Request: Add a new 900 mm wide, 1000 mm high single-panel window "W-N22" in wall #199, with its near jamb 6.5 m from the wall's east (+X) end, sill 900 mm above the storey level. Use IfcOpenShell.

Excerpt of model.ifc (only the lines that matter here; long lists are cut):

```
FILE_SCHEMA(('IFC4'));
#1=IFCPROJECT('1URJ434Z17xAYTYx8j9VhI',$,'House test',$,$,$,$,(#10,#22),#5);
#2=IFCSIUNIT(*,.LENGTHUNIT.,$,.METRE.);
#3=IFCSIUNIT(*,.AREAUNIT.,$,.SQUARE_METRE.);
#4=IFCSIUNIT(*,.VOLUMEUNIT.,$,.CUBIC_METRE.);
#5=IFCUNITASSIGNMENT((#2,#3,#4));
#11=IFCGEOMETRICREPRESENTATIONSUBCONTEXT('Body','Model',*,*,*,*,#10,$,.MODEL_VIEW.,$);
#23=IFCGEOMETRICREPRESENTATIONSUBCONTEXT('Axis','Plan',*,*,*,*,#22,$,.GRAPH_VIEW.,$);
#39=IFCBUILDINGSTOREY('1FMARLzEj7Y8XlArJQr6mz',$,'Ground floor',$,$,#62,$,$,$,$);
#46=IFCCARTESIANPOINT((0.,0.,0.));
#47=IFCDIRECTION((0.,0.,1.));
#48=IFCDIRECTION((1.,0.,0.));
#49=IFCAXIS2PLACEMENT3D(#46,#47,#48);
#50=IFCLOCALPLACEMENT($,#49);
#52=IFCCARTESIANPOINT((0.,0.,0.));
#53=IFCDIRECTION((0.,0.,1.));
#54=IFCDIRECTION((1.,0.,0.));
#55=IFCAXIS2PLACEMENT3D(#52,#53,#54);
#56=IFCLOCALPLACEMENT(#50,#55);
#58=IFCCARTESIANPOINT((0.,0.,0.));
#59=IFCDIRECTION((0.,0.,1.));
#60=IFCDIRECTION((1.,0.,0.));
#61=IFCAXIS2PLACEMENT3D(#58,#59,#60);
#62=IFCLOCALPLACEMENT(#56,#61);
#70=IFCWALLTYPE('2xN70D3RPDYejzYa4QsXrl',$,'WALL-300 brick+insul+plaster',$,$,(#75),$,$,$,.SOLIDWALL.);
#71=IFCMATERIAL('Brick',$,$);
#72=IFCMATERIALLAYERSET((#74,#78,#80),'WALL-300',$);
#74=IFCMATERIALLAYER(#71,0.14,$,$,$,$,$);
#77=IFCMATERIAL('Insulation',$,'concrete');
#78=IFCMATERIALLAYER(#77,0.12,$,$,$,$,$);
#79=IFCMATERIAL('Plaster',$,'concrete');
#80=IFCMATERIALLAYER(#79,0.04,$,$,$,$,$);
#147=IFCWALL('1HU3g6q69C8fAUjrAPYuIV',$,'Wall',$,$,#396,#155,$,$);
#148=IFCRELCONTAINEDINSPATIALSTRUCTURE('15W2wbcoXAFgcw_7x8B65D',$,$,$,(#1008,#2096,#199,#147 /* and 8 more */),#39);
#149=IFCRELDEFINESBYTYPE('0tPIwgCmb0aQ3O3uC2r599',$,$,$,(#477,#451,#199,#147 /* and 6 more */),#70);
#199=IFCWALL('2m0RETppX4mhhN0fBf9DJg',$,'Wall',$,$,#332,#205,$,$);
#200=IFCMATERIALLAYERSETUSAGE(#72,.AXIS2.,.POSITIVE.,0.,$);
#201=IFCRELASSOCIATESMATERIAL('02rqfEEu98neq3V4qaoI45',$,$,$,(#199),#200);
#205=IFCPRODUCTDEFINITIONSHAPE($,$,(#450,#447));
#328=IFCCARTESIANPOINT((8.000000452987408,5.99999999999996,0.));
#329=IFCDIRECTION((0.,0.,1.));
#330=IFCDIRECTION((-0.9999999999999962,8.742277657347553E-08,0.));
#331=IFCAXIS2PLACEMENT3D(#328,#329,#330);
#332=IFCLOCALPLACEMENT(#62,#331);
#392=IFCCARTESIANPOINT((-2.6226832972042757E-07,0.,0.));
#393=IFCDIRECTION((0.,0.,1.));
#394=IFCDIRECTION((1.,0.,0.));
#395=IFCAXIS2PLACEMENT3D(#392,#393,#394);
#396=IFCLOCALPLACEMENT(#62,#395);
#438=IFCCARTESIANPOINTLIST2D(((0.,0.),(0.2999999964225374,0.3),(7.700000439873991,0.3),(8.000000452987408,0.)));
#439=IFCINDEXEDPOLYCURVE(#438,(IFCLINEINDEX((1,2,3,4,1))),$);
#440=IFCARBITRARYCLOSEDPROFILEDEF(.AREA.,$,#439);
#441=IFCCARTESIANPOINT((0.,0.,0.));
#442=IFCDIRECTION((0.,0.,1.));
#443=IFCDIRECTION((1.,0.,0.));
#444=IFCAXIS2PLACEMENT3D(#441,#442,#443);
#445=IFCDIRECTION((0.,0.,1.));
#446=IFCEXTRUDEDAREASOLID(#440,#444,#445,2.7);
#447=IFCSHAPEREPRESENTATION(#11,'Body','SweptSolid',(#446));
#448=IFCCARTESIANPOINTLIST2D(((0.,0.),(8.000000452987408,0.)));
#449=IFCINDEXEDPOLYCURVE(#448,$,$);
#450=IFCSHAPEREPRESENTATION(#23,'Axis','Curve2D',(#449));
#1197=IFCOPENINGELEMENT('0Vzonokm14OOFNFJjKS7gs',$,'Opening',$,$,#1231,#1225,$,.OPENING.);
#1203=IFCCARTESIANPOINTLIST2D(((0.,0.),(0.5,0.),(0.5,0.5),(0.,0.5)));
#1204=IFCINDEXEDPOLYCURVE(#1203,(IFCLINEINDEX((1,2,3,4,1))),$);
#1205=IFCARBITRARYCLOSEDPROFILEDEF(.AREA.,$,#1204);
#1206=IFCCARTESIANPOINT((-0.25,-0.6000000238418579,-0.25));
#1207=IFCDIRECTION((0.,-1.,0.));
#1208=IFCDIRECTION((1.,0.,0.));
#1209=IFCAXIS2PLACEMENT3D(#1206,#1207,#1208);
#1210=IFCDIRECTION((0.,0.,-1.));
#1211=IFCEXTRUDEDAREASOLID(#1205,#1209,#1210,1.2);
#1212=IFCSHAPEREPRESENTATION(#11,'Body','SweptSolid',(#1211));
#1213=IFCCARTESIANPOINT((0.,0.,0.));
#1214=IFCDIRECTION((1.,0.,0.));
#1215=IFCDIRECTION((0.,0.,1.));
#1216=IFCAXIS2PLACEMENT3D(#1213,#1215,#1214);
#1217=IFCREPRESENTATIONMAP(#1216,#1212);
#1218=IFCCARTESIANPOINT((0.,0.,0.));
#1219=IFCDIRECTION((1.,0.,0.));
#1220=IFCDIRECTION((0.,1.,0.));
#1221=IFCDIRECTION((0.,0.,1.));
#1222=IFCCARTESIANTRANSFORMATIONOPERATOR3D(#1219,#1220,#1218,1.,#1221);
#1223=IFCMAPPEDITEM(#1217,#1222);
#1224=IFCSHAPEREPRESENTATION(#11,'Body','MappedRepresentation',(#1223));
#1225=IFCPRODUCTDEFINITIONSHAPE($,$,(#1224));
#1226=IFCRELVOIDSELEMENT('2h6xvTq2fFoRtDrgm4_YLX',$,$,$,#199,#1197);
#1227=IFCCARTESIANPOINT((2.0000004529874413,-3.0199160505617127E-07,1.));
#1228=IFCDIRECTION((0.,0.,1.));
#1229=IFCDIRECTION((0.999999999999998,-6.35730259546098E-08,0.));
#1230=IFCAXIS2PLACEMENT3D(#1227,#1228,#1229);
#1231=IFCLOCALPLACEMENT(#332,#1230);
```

```python
import numpy as np
import ifcopenshell
import ifcopenshell.api.feature
import ifcopenshell.api.geometry
import ifcopenshell.api.root
import ifcopenshell.api.spatial
import ifcopenshell.geom
import ifcopenshell.util.element
import ifcopenshell.util.placement
import ifcopenshell.util.representation
import ifcopenshell.util.shape
import ifcopenshell.util.unit

model = ifcopenshell.open("model.ifc")
unit_scale = ifcopenshell.util.unit.calculate_unit_scale(model)
settings = ifcopenshell.geom.settings()


def volume(element):
    """Net volume in cubic metres, openings subtracted."""
    shape = ifcopenshell.geom.create_shape(settings, element)
    return ifcopenshell.util.shape.get_volume(shape.geometry)


wall = model.by_guid("2m0RETppX4mhhN0fBf9DJg")
storey = ifcopenshell.util.element.get_container(wall, ifc_class="IfcBuildingStorey")
context = ifcopenshell.util.representation.get_context(model, "Model", "Body", "MODEL_VIEW")
before = volume(wall)

width, height, from_end, sill = 0.9, 1, 6.5, 0.9  # metres

# The wall runs along its own X axis, and the end named is its -X end.
wall_shape = ifcopenshell.geom.create_shape(settings, wall)
x, y, z = ifcopenshell.util.shape.get_vertices(wall_shape.geometry).T
start = x.min() + from_end
face, thickness = float(y.min()), float(y.max() - y.min())
wall_matrix = ifcopenshell.util.placement.get_local_placement(wall.ObjectPlacement)
level = ifcopenshell.util.placement.get_local_placement(storey.ObjectPlacement)[2, 3]


def in_wall(x, y):
    """Placement at x, y metres in the wall's axes, at sill height."""
    matrix = wall_matrix.copy()
    matrix[:, 3] = wall_matrix @ np.array([x / unit_scale, y / unit_scale, 0.0, 1.0])
    matrix[2, 3] = level + sill / unit_scale
    return matrix


# Opening: a box that overshoots both wall faces by 50 mm.
opening = ifcopenshell.api.root.create_entity(model, ifc_class="IfcOpeningElement", predefined_type="OPENING")
box = ifcopenshell.api.geometry.add_wall_representation(
    model, context=context, length=width, height=height, thickness=thickness + 0.1
)
ifcopenshell.api.geometry.assign_representation(model, product=opening, representation=box)
ifcopenshell.api.geometry.edit_object_placement(model, product=opening, matrix=in_wall(start, face - 0.05), is_si=False)
ifcopenshell.api.feature.add_feature(model, feature=opening, element=wall)

window = ifcopenshell.api.root.create_entity(model, ifc_class="IfcWindow", name="W-N22", predefined_type="WINDOW")
window.OverallWidth, window.OverallHeight = width / unit_scale, height / unit_scale
window.PartitioningType = "SINGLE_PANEL"
body = ifcopenshell.api.geometry.add_window_representation(
    model,
    context=context,
    overall_width=window.OverallWidth,
    overall_height=window.OverallHeight,
    partition_type="SINGLE_PANEL",
)
ifcopenshell.api.geometry.assign_representation(model, product=window, representation=body)
ifcopenshell.api.spatial.assign_container(model, products=[window], relating_structure=storey)
ifcopenshell.api.feature.add_filling(model, opening=opening, element=window)

# Centre the window in the wall's thickness.
ifcopenshell.api.geometry.edit_object_placement(model, product=window, matrix=in_wall(start, face), is_si=False)
window_shape = ifcopenshell.geom.create_shape(settings, window)
depth = ifcopenshell.util.shape.get_vertices(window_shape.geometry)[:, 1]
offset = face + thickness / 2 - (depth.min() + depth.max()) / 2
ifcopenshell.api.geometry.edit_object_placement(model, product=window, matrix=in_wall(start, offset), is_si=False)

after = volume(wall)

print(f"wall volume {before:.3f} -> {after:.3f} m3")

model.write("model-out.ifc")
```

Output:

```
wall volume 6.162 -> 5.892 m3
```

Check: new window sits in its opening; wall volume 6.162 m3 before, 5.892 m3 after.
